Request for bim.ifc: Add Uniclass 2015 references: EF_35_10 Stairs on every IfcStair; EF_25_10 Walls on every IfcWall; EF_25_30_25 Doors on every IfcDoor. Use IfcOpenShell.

First a look at what the model holds.

```python
import ifcopenshell

model = ifcopenshell.open("bim.ifc")
print(model.schema)
print("classifications:", [c.Name for c in model.by_type("IfcClassification")])
for ifc_class in ("IfcDoor", "IfcRoof", "IfcStair", "IfcWall", "IfcWindow"):
    print(ifc_class, len(model.by_type(ifc_class)))
```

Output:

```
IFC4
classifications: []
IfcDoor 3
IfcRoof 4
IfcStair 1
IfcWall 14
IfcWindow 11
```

```python
import ifcopenshell
import ifcopenshell.api.classification

model = ifcopenshell.open("bim.ifc")

system = ifcopenshell.api.classification.add_classification(model, classification="Uniclass 2015")

codes = {
    "IfcStair": ("EF_35_10", "Stairs"),
    "IfcWall": ("EF_25_10", "Walls"),
    "IfcDoor": ("EF_25_30_25", "Doors"),
}
for ifc_class, (code, name) in codes.items():
    products = model.by_type(ifc_class)
    ifcopenshell.api.classification.add_reference(
        model, products=products, classification=system, identification=code, name=name
    )
    print(code, len(products))

model.write("bim_updated.ifc")
```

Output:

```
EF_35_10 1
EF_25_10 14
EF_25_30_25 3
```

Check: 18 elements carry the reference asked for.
